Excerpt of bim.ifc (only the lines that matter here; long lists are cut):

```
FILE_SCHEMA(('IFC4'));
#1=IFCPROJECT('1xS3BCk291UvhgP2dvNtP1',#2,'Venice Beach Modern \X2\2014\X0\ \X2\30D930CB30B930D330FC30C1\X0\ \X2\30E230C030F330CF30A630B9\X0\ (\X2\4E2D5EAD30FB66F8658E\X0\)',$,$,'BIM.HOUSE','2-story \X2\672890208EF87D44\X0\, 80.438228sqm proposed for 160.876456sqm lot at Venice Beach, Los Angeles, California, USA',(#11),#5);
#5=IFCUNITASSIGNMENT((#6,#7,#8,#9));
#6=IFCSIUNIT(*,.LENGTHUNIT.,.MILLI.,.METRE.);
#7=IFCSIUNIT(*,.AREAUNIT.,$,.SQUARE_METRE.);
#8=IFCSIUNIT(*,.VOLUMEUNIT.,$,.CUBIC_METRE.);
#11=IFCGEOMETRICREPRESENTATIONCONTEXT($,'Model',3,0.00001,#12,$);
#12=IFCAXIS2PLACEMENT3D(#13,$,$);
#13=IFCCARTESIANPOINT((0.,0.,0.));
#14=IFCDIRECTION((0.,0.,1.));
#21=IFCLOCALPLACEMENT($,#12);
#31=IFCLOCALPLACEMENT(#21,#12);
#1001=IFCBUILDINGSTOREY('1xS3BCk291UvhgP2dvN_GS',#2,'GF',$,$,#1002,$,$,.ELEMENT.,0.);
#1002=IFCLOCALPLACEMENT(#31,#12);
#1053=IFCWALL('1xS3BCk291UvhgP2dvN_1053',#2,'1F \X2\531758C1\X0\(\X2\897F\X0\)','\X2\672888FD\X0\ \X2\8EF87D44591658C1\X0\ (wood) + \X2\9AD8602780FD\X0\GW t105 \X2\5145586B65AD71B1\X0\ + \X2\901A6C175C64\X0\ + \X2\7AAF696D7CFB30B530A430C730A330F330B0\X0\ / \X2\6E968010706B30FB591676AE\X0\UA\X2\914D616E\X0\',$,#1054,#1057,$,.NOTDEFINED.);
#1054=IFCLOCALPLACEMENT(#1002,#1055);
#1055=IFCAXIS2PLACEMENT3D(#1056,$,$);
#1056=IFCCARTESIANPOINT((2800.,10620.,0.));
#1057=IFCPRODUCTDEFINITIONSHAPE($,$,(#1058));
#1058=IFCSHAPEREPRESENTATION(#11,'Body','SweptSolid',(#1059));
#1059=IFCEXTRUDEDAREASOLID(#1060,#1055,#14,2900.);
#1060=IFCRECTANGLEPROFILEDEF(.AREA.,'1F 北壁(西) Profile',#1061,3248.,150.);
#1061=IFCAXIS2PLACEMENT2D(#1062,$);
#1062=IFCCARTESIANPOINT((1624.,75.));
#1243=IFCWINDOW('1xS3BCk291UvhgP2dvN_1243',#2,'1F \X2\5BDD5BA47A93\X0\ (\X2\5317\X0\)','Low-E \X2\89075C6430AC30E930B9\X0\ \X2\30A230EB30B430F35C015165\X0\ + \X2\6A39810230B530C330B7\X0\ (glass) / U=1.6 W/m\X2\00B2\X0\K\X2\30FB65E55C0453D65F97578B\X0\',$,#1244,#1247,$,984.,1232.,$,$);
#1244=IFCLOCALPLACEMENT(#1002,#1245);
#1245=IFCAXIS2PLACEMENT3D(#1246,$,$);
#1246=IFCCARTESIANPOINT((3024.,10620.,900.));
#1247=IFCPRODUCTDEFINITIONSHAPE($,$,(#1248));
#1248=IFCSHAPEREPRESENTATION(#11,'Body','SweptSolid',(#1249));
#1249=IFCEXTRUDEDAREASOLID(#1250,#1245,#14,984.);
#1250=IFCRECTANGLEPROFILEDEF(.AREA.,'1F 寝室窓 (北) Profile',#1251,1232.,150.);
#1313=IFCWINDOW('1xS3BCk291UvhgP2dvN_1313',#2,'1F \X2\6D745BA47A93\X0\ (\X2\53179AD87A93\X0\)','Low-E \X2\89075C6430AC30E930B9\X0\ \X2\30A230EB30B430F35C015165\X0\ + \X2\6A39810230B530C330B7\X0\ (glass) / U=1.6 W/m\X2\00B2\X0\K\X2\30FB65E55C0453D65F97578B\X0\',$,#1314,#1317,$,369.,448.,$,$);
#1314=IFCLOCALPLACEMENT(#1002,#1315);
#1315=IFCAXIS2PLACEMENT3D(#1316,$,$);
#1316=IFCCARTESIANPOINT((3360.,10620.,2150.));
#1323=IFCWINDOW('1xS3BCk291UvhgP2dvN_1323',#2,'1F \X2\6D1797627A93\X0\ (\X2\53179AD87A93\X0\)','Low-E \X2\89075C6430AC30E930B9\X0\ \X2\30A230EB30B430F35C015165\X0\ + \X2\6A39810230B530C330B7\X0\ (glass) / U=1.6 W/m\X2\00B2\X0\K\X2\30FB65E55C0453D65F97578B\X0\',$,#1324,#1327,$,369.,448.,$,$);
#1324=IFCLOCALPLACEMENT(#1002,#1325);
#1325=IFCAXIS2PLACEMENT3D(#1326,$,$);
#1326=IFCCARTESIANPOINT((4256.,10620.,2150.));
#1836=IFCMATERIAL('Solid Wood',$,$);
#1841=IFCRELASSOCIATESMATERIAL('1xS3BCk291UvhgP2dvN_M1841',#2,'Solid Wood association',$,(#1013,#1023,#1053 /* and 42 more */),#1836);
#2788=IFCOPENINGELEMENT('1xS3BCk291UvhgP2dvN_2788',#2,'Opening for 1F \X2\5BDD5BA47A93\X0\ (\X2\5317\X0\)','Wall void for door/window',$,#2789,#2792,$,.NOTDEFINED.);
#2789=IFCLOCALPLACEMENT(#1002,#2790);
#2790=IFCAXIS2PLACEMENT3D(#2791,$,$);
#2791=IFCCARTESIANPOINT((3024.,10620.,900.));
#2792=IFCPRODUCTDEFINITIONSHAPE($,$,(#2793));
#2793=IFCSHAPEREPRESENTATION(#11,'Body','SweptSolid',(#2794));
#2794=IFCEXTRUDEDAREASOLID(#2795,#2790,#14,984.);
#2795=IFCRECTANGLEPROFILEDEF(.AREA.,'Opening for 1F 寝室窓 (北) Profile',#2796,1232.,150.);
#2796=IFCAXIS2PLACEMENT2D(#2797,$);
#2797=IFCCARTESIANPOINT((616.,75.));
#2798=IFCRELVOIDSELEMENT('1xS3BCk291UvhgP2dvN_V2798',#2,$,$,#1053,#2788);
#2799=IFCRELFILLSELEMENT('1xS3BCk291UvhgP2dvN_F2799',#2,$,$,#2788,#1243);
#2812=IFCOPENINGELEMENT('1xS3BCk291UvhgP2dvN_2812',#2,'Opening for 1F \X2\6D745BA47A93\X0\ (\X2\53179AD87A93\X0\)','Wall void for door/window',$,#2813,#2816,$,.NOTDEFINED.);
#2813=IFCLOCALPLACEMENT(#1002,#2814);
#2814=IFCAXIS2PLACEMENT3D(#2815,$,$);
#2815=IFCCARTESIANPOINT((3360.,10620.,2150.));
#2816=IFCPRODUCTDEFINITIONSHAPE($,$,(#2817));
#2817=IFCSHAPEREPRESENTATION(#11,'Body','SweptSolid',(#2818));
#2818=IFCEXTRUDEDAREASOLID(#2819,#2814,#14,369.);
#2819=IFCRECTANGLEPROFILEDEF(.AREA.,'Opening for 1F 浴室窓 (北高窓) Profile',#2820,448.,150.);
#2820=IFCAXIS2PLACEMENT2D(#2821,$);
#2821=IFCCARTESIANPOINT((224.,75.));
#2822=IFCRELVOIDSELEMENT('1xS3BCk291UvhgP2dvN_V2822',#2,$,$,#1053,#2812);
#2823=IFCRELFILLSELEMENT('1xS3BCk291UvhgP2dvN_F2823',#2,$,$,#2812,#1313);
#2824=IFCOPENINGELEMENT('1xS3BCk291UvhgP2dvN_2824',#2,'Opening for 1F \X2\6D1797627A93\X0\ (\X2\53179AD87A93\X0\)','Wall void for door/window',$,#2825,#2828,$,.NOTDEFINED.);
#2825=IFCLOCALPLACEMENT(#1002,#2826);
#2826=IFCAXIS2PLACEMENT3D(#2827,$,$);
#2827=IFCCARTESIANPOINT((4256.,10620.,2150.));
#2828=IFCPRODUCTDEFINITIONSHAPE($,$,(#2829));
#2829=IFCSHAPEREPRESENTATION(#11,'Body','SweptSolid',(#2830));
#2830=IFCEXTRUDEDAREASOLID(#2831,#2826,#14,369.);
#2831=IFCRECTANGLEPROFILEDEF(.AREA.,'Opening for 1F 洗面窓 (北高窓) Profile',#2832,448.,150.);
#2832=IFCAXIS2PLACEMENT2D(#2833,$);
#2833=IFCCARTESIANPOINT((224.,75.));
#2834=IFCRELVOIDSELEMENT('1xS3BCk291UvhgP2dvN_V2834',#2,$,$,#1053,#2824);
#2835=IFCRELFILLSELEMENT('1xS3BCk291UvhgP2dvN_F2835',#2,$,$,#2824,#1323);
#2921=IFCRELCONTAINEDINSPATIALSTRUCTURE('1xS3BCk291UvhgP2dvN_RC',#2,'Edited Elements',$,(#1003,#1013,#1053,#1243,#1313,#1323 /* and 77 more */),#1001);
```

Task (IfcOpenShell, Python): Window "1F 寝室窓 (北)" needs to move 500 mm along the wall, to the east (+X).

```python
import ifcopenshell
import ifcopenshell.api.geometry
import ifcopenshell.util.placement

model = ifcopenshell.open("bim.ifc")

window = model.by_guid("1xS3BCk291UvhgP2dvN_1243")
opening = window.FillsVoids[0].RelatingOpeningElement
wall = opening.VoidsElements[0].RelatingBuildingElement

wall_matrix = ifcopenshell.util.placement.get_local_placement(wall.ObjectPlacement)
shift = wall_matrix[:3, 0] * 500.0
before = ifcopenshell.util.placement.get_local_placement(window.ObjectPlacement)[:3, 3].copy()

# The window is not placed relative to its opening, so move both.
for product in (opening, window):
    matrix = ifcopenshell.util.placement.get_local_placement(product.ObjectPlacement)
    matrix[:3, 3] += shift
    ifcopenshell.api.geometry.edit_object_placement(model, product=product, matrix=matrix, is_si=False)

after = ifcopenshell.util.placement.get_local_placement(window.ObjectPlacement)[:3, 3]
print("window moved by", (after - before).round(3) + 0.0)

model.write("bim_edited.ifc")
```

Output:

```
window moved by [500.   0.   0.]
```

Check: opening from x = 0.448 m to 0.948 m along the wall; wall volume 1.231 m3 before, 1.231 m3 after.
